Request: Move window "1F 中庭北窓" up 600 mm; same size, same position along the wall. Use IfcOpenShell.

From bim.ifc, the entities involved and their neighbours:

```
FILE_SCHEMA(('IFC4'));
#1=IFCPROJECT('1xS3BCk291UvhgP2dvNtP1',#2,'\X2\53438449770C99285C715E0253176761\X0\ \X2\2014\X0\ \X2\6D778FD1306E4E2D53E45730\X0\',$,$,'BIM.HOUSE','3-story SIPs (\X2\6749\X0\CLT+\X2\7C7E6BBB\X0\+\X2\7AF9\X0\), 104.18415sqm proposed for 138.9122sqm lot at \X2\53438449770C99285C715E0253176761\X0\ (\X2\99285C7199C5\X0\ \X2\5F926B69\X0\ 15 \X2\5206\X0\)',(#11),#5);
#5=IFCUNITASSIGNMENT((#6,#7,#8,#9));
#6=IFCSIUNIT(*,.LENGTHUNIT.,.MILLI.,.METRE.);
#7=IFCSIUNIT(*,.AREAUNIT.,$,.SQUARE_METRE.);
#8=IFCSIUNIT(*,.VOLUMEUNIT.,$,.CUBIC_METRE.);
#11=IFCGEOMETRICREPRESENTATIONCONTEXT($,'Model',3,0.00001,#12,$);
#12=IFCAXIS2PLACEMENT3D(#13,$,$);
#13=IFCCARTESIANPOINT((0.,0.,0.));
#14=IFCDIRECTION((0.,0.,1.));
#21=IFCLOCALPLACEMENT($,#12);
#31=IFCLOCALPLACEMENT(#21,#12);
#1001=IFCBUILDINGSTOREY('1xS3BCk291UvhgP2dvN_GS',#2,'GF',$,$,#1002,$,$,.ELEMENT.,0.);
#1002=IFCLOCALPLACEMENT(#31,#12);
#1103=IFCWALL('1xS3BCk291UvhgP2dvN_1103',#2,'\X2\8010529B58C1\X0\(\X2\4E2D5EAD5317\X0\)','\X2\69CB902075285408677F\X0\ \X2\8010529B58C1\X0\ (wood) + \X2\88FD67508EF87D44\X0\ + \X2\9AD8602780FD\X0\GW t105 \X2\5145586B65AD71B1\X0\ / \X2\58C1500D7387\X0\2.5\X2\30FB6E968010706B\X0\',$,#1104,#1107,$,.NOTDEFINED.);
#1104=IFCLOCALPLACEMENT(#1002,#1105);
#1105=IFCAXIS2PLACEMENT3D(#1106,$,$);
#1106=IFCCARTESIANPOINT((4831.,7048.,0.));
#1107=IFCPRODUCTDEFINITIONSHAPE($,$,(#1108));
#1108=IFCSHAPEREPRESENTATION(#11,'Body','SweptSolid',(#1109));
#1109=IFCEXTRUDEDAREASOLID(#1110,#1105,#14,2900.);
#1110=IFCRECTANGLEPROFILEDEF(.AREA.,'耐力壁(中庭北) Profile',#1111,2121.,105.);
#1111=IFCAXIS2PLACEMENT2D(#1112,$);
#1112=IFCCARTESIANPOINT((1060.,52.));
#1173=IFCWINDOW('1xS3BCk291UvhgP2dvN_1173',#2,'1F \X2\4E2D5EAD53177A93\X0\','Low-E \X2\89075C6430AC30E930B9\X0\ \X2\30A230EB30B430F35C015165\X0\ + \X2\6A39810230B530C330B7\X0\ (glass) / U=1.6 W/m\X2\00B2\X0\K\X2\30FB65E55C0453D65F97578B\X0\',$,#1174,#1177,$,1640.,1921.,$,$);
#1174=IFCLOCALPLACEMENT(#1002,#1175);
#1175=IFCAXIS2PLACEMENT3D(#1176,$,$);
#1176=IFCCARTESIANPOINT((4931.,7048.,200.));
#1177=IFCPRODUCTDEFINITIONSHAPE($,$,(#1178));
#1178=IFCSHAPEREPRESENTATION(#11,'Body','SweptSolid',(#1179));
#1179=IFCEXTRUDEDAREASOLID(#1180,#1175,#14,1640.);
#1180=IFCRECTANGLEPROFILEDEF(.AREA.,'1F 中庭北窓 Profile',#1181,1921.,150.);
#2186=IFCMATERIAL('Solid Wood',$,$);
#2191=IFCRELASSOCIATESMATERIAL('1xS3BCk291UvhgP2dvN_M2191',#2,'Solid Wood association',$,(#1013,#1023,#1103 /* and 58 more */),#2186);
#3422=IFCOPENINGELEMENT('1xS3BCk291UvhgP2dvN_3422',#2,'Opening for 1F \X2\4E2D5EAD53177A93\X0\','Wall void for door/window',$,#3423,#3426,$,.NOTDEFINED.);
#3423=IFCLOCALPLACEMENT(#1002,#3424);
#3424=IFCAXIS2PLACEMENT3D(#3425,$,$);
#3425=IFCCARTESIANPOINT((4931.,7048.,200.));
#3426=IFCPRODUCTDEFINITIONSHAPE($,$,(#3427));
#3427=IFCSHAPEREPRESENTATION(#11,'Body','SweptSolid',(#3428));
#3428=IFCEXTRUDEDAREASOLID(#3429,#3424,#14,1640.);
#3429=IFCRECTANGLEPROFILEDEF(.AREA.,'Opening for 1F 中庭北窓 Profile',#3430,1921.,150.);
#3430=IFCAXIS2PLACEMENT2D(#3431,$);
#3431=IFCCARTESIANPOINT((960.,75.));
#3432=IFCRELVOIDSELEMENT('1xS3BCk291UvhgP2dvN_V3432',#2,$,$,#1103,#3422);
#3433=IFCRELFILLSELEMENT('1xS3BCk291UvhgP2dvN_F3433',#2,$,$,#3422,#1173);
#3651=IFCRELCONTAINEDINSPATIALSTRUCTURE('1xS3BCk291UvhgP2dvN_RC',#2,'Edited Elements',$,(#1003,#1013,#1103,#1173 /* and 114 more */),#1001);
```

```python
import numpy as np
import ifcopenshell
import ifcopenshell.api.geometry
import ifcopenshell.util.placement
import ifcopenshell.util.unit

model = ifcopenshell.open("bim.ifc")
unit_scale = ifcopenshell.util.unit.calculate_unit_scale(model)

window = model.by_guid("1xS3BCk291UvhgP2dvN_1173")
opening = window.FillsVoids[0].RelatingOpeningElement
dz = 0.6 / unit_scale

shift = np.array([0.0, 0.0, dz])
# The window is not placed relative to its opening, so move both.
for product in (opening, window):
    matrix = ifcopenshell.util.placement.get_local_placement(product.ObjectPlacement)
    matrix[:3, 3] += shift
    ifcopenshell.api.geometry.edit_object_placement(model, product=product, matrix=matrix, is_si=False)

print(f"moved by {dz * unit_scale:+.3f} m")

model.write("bim-out.ifc")
```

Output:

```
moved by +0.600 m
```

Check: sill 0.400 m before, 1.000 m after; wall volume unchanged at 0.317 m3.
